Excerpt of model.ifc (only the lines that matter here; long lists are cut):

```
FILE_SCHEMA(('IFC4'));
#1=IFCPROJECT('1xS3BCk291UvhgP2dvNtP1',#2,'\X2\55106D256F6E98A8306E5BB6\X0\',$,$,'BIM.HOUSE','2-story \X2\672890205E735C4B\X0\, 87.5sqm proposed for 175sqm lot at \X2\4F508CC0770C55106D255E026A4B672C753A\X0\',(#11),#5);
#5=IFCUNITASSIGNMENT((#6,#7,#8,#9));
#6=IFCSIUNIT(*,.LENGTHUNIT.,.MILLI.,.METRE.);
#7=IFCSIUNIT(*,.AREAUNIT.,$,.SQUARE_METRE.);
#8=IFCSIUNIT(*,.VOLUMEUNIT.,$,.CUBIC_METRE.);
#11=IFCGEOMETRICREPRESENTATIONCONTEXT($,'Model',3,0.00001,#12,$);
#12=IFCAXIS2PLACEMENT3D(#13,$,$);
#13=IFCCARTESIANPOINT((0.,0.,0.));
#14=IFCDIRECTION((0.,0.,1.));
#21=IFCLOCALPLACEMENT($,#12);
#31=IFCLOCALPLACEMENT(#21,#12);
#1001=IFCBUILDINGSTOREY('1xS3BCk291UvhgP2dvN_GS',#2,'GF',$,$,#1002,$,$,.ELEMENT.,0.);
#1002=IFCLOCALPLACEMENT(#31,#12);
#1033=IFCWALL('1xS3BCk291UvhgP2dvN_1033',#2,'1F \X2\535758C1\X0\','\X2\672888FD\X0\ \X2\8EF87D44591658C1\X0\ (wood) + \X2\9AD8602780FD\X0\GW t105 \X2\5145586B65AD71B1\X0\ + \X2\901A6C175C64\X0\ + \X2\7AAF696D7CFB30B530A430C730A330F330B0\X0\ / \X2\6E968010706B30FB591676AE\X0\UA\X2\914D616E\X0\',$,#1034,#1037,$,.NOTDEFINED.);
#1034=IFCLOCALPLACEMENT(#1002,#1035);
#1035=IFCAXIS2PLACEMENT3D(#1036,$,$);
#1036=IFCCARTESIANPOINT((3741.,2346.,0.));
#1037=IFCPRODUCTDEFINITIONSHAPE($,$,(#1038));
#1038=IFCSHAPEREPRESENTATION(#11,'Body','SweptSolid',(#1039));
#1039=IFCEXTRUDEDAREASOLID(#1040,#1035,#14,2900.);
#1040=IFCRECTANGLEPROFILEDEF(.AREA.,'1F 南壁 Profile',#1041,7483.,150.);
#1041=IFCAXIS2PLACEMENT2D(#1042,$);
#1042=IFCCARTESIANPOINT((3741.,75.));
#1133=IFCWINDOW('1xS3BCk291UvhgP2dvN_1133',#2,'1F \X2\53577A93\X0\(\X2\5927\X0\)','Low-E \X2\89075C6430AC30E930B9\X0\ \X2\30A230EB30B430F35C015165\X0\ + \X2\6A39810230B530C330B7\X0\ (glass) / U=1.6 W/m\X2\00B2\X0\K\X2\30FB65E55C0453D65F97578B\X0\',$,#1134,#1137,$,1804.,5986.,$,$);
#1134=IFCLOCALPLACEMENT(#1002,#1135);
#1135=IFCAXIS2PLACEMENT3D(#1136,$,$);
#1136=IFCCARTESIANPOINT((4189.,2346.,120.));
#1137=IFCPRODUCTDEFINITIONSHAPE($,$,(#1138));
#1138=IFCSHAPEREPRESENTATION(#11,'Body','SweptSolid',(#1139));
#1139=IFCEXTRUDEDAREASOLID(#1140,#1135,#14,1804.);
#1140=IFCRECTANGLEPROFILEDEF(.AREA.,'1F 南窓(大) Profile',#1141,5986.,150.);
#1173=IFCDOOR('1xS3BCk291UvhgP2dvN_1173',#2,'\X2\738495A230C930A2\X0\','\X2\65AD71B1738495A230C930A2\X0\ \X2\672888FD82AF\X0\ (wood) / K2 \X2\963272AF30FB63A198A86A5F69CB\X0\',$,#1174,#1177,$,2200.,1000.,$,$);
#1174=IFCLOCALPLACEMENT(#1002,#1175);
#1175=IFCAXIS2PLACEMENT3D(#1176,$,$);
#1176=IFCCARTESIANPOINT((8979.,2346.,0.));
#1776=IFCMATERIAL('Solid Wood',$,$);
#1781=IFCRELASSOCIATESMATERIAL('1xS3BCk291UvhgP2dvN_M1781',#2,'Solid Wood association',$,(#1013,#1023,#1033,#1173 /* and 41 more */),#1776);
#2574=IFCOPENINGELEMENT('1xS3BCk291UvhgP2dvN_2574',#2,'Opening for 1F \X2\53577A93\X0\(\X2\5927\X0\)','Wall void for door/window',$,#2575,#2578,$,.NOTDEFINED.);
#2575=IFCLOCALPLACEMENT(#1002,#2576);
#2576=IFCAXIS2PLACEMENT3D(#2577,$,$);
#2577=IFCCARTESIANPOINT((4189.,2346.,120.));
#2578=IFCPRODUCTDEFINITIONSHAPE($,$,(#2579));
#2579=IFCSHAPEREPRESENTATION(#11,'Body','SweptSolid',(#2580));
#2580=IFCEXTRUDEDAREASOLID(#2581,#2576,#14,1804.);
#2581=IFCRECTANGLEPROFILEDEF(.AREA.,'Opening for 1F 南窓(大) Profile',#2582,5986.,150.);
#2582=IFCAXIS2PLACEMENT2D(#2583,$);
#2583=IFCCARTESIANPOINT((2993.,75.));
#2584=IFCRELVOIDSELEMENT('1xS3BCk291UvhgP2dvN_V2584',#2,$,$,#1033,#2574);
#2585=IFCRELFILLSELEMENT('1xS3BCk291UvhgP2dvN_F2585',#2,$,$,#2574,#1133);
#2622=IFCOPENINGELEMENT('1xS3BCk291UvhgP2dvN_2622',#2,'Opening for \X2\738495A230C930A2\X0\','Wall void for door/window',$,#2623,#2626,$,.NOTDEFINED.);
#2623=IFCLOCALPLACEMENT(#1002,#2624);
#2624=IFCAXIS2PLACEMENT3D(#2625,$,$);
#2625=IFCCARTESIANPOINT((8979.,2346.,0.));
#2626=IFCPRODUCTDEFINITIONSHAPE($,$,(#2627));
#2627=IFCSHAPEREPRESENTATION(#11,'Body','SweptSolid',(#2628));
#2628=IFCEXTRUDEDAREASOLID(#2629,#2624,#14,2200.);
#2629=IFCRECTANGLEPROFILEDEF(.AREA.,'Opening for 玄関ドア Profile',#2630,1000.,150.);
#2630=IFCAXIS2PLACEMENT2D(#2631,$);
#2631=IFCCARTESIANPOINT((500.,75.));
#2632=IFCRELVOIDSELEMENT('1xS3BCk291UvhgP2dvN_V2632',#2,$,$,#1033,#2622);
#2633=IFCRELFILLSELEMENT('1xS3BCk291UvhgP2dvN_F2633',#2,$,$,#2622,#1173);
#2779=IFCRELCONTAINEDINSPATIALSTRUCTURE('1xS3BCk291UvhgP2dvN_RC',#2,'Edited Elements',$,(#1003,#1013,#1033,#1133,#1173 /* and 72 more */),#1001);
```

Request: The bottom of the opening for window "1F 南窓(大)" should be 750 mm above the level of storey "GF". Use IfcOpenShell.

```python
import numpy as np
import ifcopenshell
import ifcopenshell.api.geometry
import ifcopenshell.geom
import ifcopenshell.util.element
import ifcopenshell.util.placement
import ifcopenshell.util.shape
import ifcopenshell.util.unit

model = ifcopenshell.open("model.ifc")
unit_scale = ifcopenshell.util.unit.calculate_unit_scale(model)

window = model.by_guid("1xS3BCk291UvhgP2dvN_1133")
opening = window.FillsVoids[0].RelatingOpeningElement
storey = ifcopenshell.util.element.get_container(window, ifc_class="IfcBuildingStorey")
level = ifcopenshell.util.placement.get_local_placement(storey.ObjectPlacement)[2, 3]

# The opening's origin need not be at the sill, so measure its lowest point.
shape = ifcopenshell.geom.create_shape(ifcopenshell.geom.settings(), opening)
bottom = ifcopenshell.util.shape.get_shape_bottom_elevation(shape, shape.geometry) / unit_scale
dz = level + 750.0 - bottom

shift = np.array([0.0, 0.0, dz])
# The window is not placed relative to its opening, so move both.
for product in (opening, window):
    matrix = ifcopenshell.util.placement.get_local_placement(product.ObjectPlacement)
    matrix[:3, 3] += shift
    ifcopenshell.api.geometry.edit_object_placement(model, product=product, matrix=matrix, is_si=False)

print(f"moved by {dz * unit_scale:+.3f} m")

model.write("model_updated.ifc")
```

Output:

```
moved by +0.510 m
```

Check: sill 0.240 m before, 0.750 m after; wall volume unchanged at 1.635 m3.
